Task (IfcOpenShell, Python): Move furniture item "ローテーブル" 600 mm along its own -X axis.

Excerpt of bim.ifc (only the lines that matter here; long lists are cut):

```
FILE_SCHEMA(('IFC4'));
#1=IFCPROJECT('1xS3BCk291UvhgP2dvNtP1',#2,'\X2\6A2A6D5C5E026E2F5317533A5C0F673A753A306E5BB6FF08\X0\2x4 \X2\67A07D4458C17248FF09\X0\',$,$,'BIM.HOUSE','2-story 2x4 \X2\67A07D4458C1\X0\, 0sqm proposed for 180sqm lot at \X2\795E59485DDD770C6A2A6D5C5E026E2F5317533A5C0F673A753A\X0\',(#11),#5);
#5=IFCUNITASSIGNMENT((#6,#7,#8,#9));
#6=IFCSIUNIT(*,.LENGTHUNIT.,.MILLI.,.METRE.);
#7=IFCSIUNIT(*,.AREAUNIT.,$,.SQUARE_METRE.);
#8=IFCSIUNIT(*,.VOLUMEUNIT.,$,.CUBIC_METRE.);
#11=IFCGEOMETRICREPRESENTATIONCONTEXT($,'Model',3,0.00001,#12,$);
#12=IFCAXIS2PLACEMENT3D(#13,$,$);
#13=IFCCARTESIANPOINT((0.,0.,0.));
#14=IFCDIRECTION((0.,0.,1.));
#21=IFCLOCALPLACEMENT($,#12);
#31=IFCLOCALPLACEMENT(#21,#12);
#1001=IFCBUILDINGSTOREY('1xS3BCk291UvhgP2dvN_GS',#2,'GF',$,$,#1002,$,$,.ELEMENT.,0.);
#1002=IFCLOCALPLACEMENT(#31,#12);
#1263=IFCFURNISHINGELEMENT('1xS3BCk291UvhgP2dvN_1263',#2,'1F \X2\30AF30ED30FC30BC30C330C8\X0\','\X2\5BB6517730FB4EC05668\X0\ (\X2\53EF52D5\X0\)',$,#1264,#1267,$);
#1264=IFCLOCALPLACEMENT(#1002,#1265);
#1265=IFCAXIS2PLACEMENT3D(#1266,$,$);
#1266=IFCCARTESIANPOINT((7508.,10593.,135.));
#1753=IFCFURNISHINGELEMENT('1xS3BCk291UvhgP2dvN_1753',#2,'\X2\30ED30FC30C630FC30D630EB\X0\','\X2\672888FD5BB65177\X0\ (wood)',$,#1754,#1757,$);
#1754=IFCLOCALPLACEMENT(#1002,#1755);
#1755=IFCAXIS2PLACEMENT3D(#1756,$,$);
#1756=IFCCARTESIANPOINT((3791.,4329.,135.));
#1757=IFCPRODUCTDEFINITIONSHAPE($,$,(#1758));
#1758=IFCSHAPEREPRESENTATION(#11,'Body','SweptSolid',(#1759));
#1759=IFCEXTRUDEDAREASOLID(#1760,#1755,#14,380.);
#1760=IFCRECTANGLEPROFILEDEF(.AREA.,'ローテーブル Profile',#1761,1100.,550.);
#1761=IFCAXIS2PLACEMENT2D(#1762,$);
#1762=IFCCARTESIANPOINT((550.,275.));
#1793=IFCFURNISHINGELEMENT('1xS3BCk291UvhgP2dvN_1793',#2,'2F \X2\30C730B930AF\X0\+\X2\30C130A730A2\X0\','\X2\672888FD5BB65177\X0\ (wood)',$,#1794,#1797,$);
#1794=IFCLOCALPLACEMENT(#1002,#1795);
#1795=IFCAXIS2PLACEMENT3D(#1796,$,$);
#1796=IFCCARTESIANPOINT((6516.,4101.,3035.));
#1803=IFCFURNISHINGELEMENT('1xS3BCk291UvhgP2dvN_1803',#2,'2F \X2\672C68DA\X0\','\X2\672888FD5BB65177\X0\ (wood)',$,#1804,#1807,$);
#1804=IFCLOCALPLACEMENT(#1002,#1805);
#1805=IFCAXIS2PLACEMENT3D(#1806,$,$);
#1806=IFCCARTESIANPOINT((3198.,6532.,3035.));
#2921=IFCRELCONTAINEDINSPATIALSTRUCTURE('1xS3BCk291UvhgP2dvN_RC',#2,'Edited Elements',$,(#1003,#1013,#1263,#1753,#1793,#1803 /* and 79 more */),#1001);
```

```python
import ifcopenshell
import ifcopenshell.api.geometry
import ifcopenshell.util.placement
import ifcopenshell.util.unit

model = ifcopenshell.open("bim.ifc")
unit_scale = ifcopenshell.util.unit.calculate_unit_scale(model)

item = model.by_guid("1xS3BCk291UvhgP2dvN_1753")
matrix = ifcopenshell.util.placement.get_local_placement(item.ObjectPlacement)
matrix[:3, 3] -= matrix[:3, 0] * 0.6 / unit_scale
ifcopenshell.api.geometry.edit_object_placement(model, product=item, matrix=matrix, is_si=False)

print(ifcopenshell.util.placement.get_local_placement(item.ObjectPlacement).round(3) + 0.0)

model.write("bim_rev.ifc")
```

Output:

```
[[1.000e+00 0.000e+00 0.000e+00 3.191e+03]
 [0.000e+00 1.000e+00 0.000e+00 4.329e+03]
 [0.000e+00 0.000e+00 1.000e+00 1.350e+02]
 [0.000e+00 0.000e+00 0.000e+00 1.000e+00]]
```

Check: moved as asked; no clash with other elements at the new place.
